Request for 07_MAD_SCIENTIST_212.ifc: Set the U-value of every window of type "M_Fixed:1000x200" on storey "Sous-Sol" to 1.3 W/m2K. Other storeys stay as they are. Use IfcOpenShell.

First a look at what the model holds.

```python
import ifcopenshell
import ifcopenshell.util.element

model = ifcopenshell.open("07_MAD_SCIENTIST_212.ifc")
print(model.schema)
storey = next(s for s in model.by_type("IfcBuildingStorey") if s.Name == "Sous-Sol")
windows = [e for e in ifcopenshell.util.element.get_decomposition(storey) if e.is_a("IfcWindow")]
seen = {}
for e in windows:
    element_type = ifcopenshell.util.element.get_type(e)
    key = (element_type.Name if element_type != e and element_type else None, ifcopenshell.util.element.get_pset(e, "Pset_WindowCommon", "ThermalTransmittance"))
    seen[key] = seen.get(key, 0) + 1
for (name, value), count in sorted(seen.items(), key=str):
    print(count, "x", name, "|", value)
```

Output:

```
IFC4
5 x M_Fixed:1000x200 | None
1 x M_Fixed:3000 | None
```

```python
import ifcopenshell
import ifcopenshell.api.pset
import ifcopenshell.util.element

model = ifcopenshell.open("07_MAD_SCIENTIST_212.ifc")

storey = next(s for s in model.by_type("IfcBuildingStorey") if s.Name == "Sous-Sol")
windows = [e for e in ifcopenshell.util.element.get_decomposition(storey) if e.is_a("IfcWindow")]

count = 0
for e in windows:
    element_type = ifcopenshell.util.element.get_type(e)
    if element_type in (None, e) or element_type.Name != "M_Fixed:1000x200":
        continue
    # add_pset returns the element's existing set when there is one.
    pset = ifcopenshell.api.pset.add_pset(model, product=e, name="Pset_WindowCommon")
    ifcopenshell.api.pset.edit_pset(model, pset=pset, properties={"ThermalTransmittance": 1.3})
    count += 1

print(count, "windows updated")

model.write("07_MAD_SCIENTIST_212_edited.ifc")
```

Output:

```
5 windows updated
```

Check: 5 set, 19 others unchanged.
